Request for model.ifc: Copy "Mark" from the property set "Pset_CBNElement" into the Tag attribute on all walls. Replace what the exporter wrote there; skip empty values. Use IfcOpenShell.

First a look at what the model holds.

```python
import ifcopenshell
import ifcopenshell.util.element

model = ifcopenshell.open("model.ifc")
print(model.schema)
walls = model.by_type("IfcWall")
print(len(walls), "walls")
for e in walls[:8]:
    source = ifcopenshell.util.element.get_pset(e, "Pset_CBNElement", "Mark")
    target = e.Tag
    print(e.id(), repr(source), repr(target), sep=" | ")
```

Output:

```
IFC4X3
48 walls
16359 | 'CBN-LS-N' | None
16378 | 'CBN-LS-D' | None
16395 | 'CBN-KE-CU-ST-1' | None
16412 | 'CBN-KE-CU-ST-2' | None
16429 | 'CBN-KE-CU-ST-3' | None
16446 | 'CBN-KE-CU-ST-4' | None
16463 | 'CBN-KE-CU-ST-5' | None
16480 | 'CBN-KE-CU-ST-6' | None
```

```python
import ifcopenshell
import ifcopenshell.util.element

model = ifcopenshell.open("model.ifc")

count = 0
for e in model.by_type("IfcWall"):
    value = ifcopenshell.util.element.get_pset(e, "Pset_CBNElement", "Mark")
    current = e.Tag
    if not value or not value.strip() or current == value:
        continue
    e.Tag = value
    count += 1

print(count, "walls updated")

model.write("model_rev.ifc")
```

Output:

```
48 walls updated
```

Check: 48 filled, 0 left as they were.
